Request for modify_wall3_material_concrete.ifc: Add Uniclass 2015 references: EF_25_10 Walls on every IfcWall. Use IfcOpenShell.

First a look at what the model holds.

```python
import ifcopenshell

model = ifcopenshell.open("modify_wall3_material_concrete.ifc")
print(model.schema)
print("classifications:", [c.Name for c in model.by_type("IfcClassification")])
for ifc_class in ("IfcDoor", "IfcRoof", "IfcStair", "IfcWall", "IfcWindow"):
    print(ifc_class, len(model.by_type(ifc_class)))
```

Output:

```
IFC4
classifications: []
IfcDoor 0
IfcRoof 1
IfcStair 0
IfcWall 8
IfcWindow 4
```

```python
import ifcopenshell
import ifcopenshell.api.classification

model = ifcopenshell.open("modify_wall3_material_concrete.ifc")

system = ifcopenshell.api.classification.add_classification(model, classification="Uniclass 2015")

codes = {
    "IfcWall": ("EF_25_10", "Walls"),
}
for ifc_class, (code, name) in codes.items():
    products = model.by_type(ifc_class)
    ifcopenshell.api.classification.add_reference(
        model, products=products, classification=system, identification=code, name=name
    )
    print(code, len(products))

model.write("modify_wall3_material_concrete_rev.ifc")
```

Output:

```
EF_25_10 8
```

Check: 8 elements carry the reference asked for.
